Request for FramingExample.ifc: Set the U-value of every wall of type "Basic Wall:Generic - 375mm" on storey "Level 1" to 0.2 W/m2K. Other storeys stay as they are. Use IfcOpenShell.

First a look at what the model holds.

```python
import ifcopenshell
import ifcopenshell.util.element

model = ifcopenshell.open("FramingExample.ifc")
print(model.schema)
storey = next(s for s in model.by_type("IfcBuildingStorey") if s.Name == "Level 1")
walls = [e for e in ifcopenshell.util.element.get_decomposition(storey) if e.is_a("IfcWall")]
seen = {}
for e in walls:
    element_type = ifcopenshell.util.element.get_type(e)
    key = (element_type.Name if element_type != e and element_type else None, ifcopenshell.util.element.get_pset(e, "Pset_WallCommon", "ThermalTransmittance"))
    seen[key] = seen.get(key, 0) + 1
for (name, value), count in sorted(seen.items(), key=str):
    print(count, "x", name, "|", value)
```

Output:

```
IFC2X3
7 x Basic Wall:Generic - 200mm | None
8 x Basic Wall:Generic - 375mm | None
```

```python
import ifcopenshell
import ifcopenshell.api.pset
import ifcopenshell.util.element

model = ifcopenshell.open("FramingExample.ifc")

storey = next(s for s in model.by_type("IfcBuildingStorey") if s.Name == "Level 1")
walls = [e for e in ifcopenshell.util.element.get_decomposition(storey) if e.is_a("IfcWall")]

count = 0
for e in walls:
    element_type = ifcopenshell.util.element.get_type(e)
    if element_type in (None, e) or element_type.Name != "Basic Wall:Generic - 375mm":
        continue
    # add_pset returns the element's existing set when there is one.
    pset = ifcopenshell.api.pset.add_pset(model, product=e, name="Pset_WallCommon")
    ifcopenshell.api.pset.edit_pset(model, pset=pset, properties={"ThermalTransmittance": 0.2})
    count += 1

print(count, "walls updated")

model.write("FramingExample_rev.ifc")
```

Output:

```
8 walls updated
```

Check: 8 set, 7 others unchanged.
